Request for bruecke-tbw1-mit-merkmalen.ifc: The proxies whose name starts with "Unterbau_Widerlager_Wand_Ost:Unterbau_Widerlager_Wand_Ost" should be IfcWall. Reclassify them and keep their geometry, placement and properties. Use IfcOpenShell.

First a look at what the model holds.

```python
import re

import ifcopenshell

model = ifcopenshell.open("bruecke-tbw1-mit-merkmalen.ifc")
print(model.schema)
seen = {}
for e in model.by_type("IfcBuildingElementProxy"):
    name = re.sub(r":\d+(:\d+)?$", "", e.Name or "")  # drop the element id that some exporters append
    seen[name] = seen.get(name, 0) + 1
for name, count in sorted(seen.items()):
    print(count, "x", name)
```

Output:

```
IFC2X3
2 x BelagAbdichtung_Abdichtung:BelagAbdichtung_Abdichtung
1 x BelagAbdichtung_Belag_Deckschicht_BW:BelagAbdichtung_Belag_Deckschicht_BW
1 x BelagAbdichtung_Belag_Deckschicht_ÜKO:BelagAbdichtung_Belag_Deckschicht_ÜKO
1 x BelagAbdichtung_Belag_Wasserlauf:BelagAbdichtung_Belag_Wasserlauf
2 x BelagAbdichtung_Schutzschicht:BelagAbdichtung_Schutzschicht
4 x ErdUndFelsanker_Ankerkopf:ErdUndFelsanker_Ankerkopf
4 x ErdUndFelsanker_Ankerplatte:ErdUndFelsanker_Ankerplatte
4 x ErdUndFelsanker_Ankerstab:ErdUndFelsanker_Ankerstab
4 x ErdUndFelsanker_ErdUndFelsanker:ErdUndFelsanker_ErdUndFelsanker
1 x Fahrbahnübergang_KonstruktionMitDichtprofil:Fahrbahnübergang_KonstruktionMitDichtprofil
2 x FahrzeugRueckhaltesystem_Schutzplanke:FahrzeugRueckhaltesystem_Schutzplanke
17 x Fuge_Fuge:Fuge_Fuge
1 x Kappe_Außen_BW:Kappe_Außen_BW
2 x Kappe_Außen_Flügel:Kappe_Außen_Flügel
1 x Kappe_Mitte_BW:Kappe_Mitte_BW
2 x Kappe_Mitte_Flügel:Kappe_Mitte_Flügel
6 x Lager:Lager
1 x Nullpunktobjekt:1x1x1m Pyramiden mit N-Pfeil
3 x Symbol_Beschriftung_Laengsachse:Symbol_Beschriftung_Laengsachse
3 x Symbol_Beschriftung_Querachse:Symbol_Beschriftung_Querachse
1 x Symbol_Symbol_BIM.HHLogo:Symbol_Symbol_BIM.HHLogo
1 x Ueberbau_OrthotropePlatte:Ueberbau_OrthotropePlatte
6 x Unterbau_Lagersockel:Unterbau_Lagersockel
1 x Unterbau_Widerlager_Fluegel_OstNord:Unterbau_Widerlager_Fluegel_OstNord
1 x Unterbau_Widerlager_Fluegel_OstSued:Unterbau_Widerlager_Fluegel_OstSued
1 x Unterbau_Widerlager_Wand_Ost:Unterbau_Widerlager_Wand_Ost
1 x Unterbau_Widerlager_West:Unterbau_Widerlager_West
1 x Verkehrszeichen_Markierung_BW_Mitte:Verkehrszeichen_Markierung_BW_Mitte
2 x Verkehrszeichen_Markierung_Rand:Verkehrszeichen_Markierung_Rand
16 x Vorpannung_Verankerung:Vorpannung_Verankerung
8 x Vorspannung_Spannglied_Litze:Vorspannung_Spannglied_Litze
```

```python
import ifcopenshell
import ifcopenshell.api.root

model = ifcopenshell.open("bruecke-tbw1-mit-merkmalen.ifc")

proxies = [e.id() for e in model.by_type("IfcBuildingElementProxy") if (e.Name or "").startswith("Unterbau_Widerlager_Wand_Ost:Unterbau_Widerlager_Wand_Ost")]
for step_id in proxies:
    proxy = model.by_id(step_id)
    # Reclassifying a typed element also reclassifies its type and the type's other occurrences.
    if proxy.is_a("IfcBuildingElementProxy"):
        ifcopenshell.api.root.reassign_class(model, product=proxy, ifc_class="IfcWall")

print(sum(model.by_id(i).is_a("IfcWall") for i in proxies), "reclassified")

model.write("bruecke-tbw1-mit-merkmalen_v2.ifc")
```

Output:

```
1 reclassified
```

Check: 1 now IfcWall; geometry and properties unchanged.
